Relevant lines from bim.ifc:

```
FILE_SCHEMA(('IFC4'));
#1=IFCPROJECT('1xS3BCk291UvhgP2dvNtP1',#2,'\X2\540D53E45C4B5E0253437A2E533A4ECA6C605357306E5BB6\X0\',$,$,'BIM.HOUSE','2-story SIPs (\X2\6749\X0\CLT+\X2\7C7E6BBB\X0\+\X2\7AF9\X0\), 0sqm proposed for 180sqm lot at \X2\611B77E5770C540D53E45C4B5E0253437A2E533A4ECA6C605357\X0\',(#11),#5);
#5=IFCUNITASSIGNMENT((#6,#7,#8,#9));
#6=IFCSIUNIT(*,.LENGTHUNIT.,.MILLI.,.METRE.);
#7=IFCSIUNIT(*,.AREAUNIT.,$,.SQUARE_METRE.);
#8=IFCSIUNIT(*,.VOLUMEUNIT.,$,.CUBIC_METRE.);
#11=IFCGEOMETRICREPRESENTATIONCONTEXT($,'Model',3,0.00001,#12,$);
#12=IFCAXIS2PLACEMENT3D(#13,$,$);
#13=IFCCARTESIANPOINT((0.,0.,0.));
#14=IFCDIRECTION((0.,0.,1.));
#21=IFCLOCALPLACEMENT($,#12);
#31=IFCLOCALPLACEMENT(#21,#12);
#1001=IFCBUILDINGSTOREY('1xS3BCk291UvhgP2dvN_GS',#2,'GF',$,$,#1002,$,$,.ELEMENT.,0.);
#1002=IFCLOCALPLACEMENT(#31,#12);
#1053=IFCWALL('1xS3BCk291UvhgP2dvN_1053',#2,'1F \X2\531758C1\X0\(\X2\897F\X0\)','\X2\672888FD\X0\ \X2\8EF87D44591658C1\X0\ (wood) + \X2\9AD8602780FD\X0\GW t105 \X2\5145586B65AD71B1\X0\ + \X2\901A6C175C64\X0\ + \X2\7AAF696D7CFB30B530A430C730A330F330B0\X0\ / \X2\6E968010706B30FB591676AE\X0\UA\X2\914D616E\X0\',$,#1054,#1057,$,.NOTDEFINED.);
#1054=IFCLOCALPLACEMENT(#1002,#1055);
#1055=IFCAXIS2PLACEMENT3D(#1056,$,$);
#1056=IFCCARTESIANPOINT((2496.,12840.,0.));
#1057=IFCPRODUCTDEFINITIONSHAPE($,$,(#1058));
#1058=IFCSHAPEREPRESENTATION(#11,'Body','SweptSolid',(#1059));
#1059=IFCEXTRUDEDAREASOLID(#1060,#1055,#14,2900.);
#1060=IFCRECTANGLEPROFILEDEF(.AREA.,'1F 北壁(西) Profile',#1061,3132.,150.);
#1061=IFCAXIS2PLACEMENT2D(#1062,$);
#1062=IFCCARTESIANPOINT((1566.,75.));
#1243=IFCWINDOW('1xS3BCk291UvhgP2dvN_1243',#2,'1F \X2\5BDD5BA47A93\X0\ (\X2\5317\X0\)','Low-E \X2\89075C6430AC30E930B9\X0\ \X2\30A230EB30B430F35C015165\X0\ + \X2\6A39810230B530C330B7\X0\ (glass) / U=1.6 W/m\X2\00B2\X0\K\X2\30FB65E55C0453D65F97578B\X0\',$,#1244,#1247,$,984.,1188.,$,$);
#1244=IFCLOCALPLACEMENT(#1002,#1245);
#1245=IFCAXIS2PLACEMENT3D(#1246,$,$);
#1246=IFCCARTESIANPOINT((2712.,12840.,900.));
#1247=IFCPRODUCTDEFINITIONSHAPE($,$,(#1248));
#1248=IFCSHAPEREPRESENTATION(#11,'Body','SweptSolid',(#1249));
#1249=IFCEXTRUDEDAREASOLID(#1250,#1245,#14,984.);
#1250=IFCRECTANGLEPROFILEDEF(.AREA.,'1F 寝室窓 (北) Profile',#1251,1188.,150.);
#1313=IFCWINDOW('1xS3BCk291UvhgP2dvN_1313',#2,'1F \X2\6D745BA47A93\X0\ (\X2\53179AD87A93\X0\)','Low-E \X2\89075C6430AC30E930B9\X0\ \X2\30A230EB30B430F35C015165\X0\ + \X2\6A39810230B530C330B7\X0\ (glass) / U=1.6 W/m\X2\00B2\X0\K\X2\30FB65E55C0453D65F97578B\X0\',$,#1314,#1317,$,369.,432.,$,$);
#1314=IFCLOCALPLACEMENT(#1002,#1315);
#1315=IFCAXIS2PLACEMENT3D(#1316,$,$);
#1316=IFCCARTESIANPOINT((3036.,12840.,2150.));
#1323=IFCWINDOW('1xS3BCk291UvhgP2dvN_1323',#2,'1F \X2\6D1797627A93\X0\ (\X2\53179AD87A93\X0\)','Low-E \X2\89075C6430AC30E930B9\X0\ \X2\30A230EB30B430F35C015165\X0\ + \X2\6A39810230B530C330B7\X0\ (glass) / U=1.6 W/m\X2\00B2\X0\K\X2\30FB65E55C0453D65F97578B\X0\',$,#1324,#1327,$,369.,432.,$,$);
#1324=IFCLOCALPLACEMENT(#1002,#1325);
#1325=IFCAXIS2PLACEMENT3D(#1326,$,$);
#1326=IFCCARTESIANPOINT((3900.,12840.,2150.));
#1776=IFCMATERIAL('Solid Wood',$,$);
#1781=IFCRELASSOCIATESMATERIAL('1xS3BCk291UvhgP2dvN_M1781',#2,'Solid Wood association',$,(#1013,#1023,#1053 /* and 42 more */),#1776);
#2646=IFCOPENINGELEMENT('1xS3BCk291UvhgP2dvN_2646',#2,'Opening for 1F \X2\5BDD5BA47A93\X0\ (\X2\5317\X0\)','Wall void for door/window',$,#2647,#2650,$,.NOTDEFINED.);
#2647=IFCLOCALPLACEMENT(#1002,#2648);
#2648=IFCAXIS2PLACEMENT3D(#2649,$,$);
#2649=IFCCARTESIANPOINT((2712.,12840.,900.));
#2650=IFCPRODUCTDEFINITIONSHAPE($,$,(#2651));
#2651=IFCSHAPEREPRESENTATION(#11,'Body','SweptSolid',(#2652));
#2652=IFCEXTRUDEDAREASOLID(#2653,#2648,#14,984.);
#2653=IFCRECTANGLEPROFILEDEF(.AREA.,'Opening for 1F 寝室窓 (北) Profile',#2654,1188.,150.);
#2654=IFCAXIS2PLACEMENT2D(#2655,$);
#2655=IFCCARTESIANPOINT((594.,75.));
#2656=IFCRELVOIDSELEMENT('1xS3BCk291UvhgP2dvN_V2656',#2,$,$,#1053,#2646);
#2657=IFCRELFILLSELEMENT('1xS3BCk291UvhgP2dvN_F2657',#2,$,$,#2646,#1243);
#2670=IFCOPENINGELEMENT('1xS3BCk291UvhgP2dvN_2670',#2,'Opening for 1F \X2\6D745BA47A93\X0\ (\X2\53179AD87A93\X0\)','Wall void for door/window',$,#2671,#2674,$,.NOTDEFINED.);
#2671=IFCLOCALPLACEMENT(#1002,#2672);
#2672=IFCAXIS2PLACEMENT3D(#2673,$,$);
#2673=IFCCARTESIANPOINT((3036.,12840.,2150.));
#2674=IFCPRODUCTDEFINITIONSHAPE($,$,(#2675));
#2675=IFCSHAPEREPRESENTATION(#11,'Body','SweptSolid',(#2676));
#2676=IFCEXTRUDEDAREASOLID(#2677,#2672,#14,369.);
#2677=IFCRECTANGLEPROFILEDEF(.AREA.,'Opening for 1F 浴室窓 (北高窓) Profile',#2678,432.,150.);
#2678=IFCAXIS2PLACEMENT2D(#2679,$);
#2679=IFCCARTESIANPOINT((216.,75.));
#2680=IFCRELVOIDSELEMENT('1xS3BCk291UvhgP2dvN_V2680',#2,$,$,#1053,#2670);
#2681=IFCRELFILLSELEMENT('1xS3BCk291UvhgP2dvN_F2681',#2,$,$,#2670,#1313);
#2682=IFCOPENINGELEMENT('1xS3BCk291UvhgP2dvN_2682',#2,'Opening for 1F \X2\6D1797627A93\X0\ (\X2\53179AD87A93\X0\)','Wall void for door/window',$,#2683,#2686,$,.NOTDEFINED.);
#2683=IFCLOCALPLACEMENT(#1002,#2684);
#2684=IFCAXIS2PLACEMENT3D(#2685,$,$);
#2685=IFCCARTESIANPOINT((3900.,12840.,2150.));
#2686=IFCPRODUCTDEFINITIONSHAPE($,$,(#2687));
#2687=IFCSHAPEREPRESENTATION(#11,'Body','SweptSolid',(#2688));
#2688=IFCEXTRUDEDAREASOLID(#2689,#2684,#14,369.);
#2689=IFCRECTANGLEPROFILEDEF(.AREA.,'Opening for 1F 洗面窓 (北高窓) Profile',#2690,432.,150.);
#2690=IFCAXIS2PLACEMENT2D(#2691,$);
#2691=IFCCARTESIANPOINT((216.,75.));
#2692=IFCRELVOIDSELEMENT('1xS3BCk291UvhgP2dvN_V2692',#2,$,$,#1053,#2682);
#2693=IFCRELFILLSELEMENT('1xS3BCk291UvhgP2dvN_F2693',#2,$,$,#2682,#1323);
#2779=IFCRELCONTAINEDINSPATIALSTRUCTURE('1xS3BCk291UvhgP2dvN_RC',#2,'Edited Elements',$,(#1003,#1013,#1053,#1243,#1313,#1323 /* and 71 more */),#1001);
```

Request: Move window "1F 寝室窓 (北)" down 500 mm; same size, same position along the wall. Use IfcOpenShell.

```python
import numpy as np
import ifcopenshell
import ifcopenshell.api.geometry
import ifcopenshell.util.placement
import ifcopenshell.util.unit

model = ifcopenshell.open("bim.ifc")
unit_scale = ifcopenshell.util.unit.calculate_unit_scale(model)

window = model.by_id(1243)
opening = window.FillsVoids[0].RelatingOpeningElement
dz = -500.0

shift = np.array([0.0, 0.0, dz])
# The window is not placed relative to its opening, so move both.
for product in (opening, window):
    matrix = ifcopenshell.util.placement.get_local_placement(product.ObjectPlacement)
    matrix[:3, 3] += shift
    ifcopenshell.api.geometry.edit_object_placement(model, product=product, matrix=matrix, is_si=False)

print(f"moved by {dz * unit_scale:+.3f} m")

model.write("bim_rev.ifc")
```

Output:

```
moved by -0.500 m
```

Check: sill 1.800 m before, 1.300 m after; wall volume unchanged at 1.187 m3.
